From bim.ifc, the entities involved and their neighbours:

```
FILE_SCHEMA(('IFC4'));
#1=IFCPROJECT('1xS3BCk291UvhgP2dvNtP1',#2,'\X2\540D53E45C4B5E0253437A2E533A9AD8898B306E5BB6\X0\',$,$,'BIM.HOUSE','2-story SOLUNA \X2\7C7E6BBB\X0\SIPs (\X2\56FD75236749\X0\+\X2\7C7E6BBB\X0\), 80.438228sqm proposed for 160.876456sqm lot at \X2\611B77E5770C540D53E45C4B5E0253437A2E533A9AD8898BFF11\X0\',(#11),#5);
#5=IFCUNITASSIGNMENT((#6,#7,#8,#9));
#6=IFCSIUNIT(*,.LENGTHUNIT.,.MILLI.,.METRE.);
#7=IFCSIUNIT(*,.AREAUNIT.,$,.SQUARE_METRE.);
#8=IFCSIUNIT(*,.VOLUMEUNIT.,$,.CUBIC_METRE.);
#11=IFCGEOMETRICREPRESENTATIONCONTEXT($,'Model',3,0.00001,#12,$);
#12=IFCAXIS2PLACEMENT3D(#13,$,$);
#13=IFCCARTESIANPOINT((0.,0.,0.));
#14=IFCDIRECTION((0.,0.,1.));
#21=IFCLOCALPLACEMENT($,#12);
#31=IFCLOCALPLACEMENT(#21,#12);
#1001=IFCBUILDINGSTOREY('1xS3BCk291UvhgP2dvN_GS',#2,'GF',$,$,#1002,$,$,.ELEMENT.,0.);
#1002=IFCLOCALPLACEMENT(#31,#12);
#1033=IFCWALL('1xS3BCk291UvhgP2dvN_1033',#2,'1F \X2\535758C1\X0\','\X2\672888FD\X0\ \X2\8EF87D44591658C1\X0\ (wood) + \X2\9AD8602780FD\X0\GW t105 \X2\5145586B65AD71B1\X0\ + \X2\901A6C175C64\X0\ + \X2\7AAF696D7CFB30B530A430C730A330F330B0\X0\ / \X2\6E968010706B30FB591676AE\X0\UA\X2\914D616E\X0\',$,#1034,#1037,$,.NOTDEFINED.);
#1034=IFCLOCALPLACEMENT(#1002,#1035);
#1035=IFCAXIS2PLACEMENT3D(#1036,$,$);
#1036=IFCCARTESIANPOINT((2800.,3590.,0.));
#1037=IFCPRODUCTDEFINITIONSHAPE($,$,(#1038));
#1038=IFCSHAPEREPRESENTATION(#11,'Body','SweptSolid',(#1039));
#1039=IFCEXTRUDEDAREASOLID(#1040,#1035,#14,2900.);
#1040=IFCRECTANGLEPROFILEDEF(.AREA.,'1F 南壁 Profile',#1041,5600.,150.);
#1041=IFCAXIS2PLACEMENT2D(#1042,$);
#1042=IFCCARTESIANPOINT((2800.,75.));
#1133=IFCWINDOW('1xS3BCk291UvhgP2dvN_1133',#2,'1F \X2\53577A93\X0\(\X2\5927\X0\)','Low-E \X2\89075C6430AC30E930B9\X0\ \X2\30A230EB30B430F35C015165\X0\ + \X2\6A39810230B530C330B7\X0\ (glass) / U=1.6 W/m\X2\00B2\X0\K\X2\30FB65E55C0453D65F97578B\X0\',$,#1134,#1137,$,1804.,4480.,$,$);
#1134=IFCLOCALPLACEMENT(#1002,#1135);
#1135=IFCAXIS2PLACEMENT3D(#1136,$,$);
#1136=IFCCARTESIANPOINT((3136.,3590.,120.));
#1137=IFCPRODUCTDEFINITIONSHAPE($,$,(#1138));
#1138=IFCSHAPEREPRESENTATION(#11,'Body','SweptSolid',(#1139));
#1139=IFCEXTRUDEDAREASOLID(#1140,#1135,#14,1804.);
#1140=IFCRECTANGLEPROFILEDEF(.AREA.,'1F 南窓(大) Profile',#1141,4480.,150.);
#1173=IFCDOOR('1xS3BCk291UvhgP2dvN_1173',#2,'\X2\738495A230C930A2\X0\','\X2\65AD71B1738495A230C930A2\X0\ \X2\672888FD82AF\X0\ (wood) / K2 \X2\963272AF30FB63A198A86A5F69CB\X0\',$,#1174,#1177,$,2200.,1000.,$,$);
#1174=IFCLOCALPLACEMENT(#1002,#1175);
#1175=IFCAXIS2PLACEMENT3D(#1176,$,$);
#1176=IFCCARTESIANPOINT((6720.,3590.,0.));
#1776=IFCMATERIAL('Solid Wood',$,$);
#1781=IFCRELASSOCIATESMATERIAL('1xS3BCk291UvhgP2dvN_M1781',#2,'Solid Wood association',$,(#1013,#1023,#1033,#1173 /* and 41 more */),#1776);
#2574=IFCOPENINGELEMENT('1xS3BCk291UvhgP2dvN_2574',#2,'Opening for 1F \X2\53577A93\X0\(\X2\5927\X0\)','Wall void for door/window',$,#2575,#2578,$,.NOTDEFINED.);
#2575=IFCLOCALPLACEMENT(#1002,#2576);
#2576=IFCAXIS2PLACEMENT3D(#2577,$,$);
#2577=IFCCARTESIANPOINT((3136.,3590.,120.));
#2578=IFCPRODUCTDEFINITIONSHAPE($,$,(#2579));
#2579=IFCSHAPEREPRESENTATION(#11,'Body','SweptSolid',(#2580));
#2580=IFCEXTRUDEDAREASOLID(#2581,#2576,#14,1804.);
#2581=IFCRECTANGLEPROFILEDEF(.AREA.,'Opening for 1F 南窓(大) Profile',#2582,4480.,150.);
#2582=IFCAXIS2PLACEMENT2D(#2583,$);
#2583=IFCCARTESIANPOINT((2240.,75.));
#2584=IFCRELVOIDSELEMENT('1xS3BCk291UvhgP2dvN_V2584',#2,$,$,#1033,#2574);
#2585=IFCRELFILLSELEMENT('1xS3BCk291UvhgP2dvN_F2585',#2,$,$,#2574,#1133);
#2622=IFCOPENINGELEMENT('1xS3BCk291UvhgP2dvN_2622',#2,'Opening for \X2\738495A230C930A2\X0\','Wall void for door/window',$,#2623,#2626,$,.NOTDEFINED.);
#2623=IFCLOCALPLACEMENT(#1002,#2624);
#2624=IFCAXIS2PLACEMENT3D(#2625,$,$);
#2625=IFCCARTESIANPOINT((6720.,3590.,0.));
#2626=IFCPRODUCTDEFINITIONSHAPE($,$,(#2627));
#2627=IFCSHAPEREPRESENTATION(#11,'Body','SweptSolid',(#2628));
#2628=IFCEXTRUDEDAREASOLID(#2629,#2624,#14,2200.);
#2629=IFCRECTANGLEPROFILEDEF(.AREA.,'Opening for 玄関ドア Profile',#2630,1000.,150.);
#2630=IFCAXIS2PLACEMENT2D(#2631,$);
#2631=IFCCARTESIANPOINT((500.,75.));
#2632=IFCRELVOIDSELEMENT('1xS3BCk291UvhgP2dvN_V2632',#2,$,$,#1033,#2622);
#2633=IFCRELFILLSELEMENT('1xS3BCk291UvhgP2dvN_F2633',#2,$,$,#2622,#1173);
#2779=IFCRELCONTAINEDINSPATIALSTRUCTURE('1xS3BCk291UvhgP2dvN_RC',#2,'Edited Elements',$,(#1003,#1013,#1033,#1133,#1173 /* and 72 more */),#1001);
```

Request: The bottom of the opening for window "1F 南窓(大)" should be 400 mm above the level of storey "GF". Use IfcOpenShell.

```python
import numpy as np
import ifcopenshell
import ifcopenshell.api.geometry
import ifcopenshell.geom
import ifcopenshell.util.element
import ifcopenshell.util.placement
import ifcopenshell.util.shape
import ifcopenshell.util.unit

model = ifcopenshell.open("bim.ifc")
unit_scale = ifcopenshell.util.unit.calculate_unit_scale(model)

window = model.by_guid("1xS3BCk291UvhgP2dvN_1133")
opening = window.FillsVoids[0].RelatingOpeningElement
storey = ifcopenshell.util.element.get_container(window, ifc_class="IfcBuildingStorey")
level = ifcopenshell.util.placement.get_local_placement(storey.ObjectPlacement)[2, 3]

# The opening's origin need not be at the sill, so measure its lowest point.
shape = ifcopenshell.geom.create_shape(ifcopenshell.geom.settings(), opening)
bottom = ifcopenshell.util.shape.get_shape_bottom_elevation(shape, shape.geometry) / unit_scale
dz = level + 0.4 / unit_scale - bottom

shift = np.array([0.0, 0.0, dz])
# The window is not placed relative to its opening, so move both.
for product in (opening, window):
    matrix = ifcopenshell.util.placement.get_local_placement(product.ObjectPlacement)
    matrix[:3, 3] += shift
    ifcopenshell.api.geometry.edit_object_placement(model, product=product, matrix=matrix, is_si=False)

print(f"moved by {dz * unit_scale:+.3f} m")

model.write("bim_rev.ifc")
```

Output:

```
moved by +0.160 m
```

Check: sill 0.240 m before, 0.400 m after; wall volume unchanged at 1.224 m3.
